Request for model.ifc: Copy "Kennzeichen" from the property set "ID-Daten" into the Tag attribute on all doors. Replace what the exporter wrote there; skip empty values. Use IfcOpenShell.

First a look at what the model holds.

```python
import ifcopenshell
import ifcopenshell.util.element

model = ifcopenshell.open("model.ifc")
print(model.schema)
doors = model.by_type("IfcDoor")
print(len(doors), "doors")
for e in doors[:8]:
    source = ifcopenshell.util.element.get_pset(e, "ID-Daten", "Kennzeichen")
    target = e.Tag
    print(e.id(), repr(source), repr(target), sep=" | ")
```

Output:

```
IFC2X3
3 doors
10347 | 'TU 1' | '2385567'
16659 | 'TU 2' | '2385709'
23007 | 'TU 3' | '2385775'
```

```python
import ifcopenshell
import ifcopenshell.util.element

model = ifcopenshell.open("model.ifc")

count = 0
for e in model.by_type("IfcDoor"):
    value = ifcopenshell.util.element.get_pset(e, "ID-Daten", "Kennzeichen")
    current = e.Tag
    if not value or not value.strip() or current == value:
        continue
    e.Tag = value
    count += 1

print(count, "doors updated")

model.write("model_rev.ifc")
```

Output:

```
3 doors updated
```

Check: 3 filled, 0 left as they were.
